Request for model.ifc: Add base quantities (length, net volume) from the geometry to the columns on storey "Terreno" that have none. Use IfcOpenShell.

First a look at what the model holds.

```python
import ifcopenshell
import ifcopenshell.util.element
import ifcopenshell.util.unit

model = ifcopenshell.open("model.ifc")
print(model.schema)
for unit_type in ("LENGTHUNIT", "AREAUNIT", "VOLUMEUNIT"):
    print(unit_type, ifcopenshell.util.unit.calculate_unit_scale(model, unit_type))
storey = next(s for s in model.by_type("IfcBuildingStorey") if s.Name == "Terreno")
columns = [e for e in ifcopenshell.util.element.get_decomposition(storey) if e.is_a("IfcColumn")]
for e in sorted(columns, key=lambda e: e.id()):
    print(e.id(), e.is_a(), e.Name, list(ifcopenshell.util.element.get_psets(e, qtos_only=True)), sep=" | ")
```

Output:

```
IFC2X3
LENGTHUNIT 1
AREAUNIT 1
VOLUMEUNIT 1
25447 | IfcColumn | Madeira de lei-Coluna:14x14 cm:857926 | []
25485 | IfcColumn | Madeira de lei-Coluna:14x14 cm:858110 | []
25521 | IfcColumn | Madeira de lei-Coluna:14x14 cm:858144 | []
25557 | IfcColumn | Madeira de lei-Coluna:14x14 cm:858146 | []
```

```python
import ifcopenshell
import ifcopenshell.api.pset
import ifcopenshell.geom
import ifcopenshell.util.element
import ifcopenshell.util.shape
import ifcopenshell.util.unit

model = ifcopenshell.open("model.ifc")
unit_scale = ifcopenshell.util.unit.calculate_unit_scale(model)
volume_scale = ifcopenshell.util.unit.calculate_unit_scale(model, "VOLUMEUNIT")
settings = ifcopenshell.geom.settings()

storey = next(s for s in model.by_type("IfcBuildingStorey") if s.Name == "Terreno")
columns = [e for e in ifcopenshell.util.element.get_decomposition(storey) if e.is_a("IfcColumn")]

for e in sorted(columns, key=lambda e: e.id()):
    if ifcopenshell.util.element.get_psets(e, qtos_only=True, should_inherit=False):
        continue
    # Geometry comes back in metres, in the element's own axes.
    shape = ifcopenshell.geom.create_shape(settings, e)
    values = {
        "Length": ifcopenshell.util.shape.get_z(shape.geometry) / unit_scale,
        "NetVolume": ifcopenshell.util.shape.get_volume(shape.geometry) / volume_scale,
    }
    qto = ifcopenshell.api.pset.add_qto(model, product=e, name="BaseQuantities")
    ifcopenshell.api.pset.edit_qto(model, qto=qto, properties=values)
    print(e.id(), {k: round(v, 3) for k, v in values.items()})

model.write("model_v2.ifc")
```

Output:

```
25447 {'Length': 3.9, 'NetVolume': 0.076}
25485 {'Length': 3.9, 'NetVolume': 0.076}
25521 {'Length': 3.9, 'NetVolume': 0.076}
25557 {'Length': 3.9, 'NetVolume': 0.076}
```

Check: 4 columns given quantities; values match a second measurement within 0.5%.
